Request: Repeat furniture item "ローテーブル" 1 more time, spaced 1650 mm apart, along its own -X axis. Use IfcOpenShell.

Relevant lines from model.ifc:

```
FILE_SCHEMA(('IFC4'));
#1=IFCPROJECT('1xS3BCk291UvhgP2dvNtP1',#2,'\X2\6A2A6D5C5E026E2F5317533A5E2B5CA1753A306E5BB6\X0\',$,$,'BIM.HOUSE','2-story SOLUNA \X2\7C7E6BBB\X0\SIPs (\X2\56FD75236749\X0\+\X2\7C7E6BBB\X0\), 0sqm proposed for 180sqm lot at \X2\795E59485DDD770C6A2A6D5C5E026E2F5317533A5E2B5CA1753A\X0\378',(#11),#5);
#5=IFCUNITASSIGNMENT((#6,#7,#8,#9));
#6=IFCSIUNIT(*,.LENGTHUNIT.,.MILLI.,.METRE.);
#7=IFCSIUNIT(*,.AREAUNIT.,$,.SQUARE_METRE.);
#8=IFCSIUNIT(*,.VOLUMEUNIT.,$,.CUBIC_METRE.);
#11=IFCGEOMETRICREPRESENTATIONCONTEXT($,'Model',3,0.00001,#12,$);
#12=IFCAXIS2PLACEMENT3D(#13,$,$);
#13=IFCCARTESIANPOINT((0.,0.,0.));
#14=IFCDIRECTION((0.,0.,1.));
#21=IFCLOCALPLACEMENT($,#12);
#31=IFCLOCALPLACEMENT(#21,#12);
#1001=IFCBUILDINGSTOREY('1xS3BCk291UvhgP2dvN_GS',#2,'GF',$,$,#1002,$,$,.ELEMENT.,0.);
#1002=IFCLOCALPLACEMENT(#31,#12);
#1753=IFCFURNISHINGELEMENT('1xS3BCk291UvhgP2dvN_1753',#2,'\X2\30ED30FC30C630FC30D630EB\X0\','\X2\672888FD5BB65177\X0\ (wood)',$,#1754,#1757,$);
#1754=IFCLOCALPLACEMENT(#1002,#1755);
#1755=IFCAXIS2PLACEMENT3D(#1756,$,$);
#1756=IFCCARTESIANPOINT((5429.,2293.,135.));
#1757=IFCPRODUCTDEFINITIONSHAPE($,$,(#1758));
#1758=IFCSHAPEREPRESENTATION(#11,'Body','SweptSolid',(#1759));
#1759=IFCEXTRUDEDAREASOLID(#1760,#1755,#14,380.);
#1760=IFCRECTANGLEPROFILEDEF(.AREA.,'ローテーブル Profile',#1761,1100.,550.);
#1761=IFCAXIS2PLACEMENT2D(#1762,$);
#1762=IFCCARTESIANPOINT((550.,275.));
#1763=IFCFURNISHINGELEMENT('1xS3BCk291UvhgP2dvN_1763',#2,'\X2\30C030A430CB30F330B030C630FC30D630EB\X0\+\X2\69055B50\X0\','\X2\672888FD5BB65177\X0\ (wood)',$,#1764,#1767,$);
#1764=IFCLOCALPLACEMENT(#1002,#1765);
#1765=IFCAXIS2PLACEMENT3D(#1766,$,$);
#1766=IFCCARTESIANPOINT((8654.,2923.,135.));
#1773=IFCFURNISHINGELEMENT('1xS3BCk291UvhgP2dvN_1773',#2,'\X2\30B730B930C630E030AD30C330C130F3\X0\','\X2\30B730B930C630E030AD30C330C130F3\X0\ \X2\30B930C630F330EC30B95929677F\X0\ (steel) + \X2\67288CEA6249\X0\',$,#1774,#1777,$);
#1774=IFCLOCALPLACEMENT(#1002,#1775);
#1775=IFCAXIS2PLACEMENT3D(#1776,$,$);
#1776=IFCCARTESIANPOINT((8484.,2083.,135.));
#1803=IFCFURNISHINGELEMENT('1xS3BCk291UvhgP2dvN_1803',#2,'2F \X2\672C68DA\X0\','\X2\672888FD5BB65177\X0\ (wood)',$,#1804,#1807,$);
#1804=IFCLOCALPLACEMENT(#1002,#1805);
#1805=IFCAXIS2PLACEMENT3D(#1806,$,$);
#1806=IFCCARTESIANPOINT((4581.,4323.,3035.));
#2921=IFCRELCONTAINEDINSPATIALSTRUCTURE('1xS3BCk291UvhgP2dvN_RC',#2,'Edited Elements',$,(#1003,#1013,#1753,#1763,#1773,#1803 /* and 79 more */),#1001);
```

```python
import ifcopenshell
import ifcopenshell.api.geometry
import ifcopenshell.api.root
import ifcopenshell.util.element
import ifcopenshell.util.placement
import ifcopenshell.util.unit

model = ifcopenshell.open("model.ifc")
unit_scale = ifcopenshell.util.unit.calculate_unit_scale(model)


def reuse_history(source, copy):
    """copy_class also copies each property set's owner history, people and application; keep the originals."""
    for rel in copy.IsDefinedBy:
        if rel.is_a("IfcRelDefinesByProperties") and (history := rel.RelatingPropertyDefinition.OwnerHistory):
            rel.RelatingPropertyDefinition.OwnerHistory = source.OwnerHistory
            ifcopenshell.util.element.remove_deep2(model, history)


source = model.by_guid("1xS3BCk291UvhgP2dvN_1753")
base = ifcopenshell.util.placement.get_local_placement(source.ObjectPlacement)
step = -base[:3, 0] * 1.65 / unit_scale

for i in range(1, 2):
    copy = ifcopenshell.api.root.copy_class(model, product=source)
    copy.Representation = ifcopenshell.util.element.copy_deep(
        model, source.Representation, exclude=["IfcGeometricRepresentationContext", "IfcRepresentationMap"]
    )
    reuse_history(source, copy)
    matrix = base.copy()
    matrix[:3, 3] += i * step
    print("added at", matrix[:3, 3].round(3) + 0.0)
    ifcopenshell.api.geometry.edit_object_placement(model, product=copy, matrix=matrix, is_si=False)

model.write("model_updated.ifc")
```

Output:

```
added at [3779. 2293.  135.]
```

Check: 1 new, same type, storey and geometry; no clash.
